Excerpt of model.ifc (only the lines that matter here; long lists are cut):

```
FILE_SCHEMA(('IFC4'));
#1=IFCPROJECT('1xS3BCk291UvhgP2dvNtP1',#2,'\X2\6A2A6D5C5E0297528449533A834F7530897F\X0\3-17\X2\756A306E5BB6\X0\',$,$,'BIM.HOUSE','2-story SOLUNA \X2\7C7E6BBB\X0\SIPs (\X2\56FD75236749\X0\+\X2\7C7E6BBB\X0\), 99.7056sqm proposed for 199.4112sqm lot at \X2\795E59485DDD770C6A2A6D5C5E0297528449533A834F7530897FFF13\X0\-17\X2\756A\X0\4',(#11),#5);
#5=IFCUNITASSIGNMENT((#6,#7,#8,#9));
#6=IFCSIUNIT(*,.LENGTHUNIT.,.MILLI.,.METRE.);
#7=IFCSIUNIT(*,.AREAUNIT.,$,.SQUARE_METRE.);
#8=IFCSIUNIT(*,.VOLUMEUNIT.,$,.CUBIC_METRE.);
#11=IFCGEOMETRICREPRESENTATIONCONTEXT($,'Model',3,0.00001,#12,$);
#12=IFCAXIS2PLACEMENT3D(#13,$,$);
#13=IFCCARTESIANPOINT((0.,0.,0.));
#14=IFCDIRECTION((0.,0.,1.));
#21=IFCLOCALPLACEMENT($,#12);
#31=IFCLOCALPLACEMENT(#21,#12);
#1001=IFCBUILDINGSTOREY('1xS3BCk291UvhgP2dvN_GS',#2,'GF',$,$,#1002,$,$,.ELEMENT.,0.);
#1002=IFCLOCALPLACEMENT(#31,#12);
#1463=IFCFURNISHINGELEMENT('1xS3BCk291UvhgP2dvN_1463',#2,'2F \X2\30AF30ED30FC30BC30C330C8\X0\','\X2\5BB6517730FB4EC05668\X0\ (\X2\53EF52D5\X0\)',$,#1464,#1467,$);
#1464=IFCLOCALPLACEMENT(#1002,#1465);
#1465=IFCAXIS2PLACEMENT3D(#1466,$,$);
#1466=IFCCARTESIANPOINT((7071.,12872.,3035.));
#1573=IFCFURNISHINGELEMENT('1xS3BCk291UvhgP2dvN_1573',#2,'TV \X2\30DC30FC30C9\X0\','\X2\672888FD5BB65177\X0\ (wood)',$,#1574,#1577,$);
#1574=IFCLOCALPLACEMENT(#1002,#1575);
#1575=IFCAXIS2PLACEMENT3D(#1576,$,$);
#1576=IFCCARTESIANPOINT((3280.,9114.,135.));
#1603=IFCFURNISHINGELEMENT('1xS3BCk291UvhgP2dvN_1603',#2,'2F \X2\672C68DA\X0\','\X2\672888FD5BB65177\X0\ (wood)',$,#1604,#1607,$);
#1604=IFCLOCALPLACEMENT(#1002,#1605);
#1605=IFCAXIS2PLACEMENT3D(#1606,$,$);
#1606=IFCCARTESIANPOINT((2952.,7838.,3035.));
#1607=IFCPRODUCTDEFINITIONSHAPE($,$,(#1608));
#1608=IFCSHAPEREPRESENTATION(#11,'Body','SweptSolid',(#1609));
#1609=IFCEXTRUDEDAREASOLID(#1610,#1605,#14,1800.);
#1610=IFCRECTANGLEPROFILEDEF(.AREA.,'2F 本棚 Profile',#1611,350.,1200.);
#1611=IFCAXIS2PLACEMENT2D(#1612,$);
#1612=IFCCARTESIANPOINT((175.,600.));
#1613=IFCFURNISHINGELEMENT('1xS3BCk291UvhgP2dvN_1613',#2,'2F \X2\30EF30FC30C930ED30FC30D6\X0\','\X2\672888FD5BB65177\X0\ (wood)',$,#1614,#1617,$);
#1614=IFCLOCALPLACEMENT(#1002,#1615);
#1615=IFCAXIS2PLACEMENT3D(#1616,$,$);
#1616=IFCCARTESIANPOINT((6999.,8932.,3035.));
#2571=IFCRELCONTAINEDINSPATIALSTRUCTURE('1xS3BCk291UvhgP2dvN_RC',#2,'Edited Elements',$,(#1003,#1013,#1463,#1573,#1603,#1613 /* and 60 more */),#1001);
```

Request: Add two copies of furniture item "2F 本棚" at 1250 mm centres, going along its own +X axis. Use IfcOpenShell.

```python
import ifcopenshell
import ifcopenshell.api.geometry
import ifcopenshell.api.root
import ifcopenshell.util.element
import ifcopenshell.util.placement
import ifcopenshell.util.unit

model = ifcopenshell.open("model.ifc")
unit_scale = ifcopenshell.util.unit.calculate_unit_scale(model)


def reuse_history(source, copy):
    """copy_class also copies each property set's owner history, people and application; keep the originals."""
    for rel in copy.IsDefinedBy:
        if rel.is_a("IfcRelDefinesByProperties") and (history := rel.RelatingPropertyDefinition.OwnerHistory):
            rel.RelatingPropertyDefinition.OwnerHistory = source.OwnerHistory
            ifcopenshell.util.element.remove_deep2(model, history)


source = model.by_guid("1xS3BCk291UvhgP2dvN_1603")
base = ifcopenshell.util.placement.get_local_placement(source.ObjectPlacement)
step = base[:3, 0] * 1.25 / unit_scale

for i in range(1, 3):
    copy = ifcopenshell.api.root.copy_class(model, product=source)
    copy.Representation = ifcopenshell.util.element.copy_deep(
        model, source.Representation, exclude=["IfcGeometricRepresentationContext", "IfcRepresentationMap"]
    )
    reuse_history(source, copy)
    matrix = base.copy()
    matrix[:3, 3] += i * step
    print("added at", matrix[:3, 3].round(3) + 0.0)
    ifcopenshell.api.geometry.edit_object_placement(model, product=copy, matrix=matrix, is_si=False)

model.write("model_rev.ifc")
```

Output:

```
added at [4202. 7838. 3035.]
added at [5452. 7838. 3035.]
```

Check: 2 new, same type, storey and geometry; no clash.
